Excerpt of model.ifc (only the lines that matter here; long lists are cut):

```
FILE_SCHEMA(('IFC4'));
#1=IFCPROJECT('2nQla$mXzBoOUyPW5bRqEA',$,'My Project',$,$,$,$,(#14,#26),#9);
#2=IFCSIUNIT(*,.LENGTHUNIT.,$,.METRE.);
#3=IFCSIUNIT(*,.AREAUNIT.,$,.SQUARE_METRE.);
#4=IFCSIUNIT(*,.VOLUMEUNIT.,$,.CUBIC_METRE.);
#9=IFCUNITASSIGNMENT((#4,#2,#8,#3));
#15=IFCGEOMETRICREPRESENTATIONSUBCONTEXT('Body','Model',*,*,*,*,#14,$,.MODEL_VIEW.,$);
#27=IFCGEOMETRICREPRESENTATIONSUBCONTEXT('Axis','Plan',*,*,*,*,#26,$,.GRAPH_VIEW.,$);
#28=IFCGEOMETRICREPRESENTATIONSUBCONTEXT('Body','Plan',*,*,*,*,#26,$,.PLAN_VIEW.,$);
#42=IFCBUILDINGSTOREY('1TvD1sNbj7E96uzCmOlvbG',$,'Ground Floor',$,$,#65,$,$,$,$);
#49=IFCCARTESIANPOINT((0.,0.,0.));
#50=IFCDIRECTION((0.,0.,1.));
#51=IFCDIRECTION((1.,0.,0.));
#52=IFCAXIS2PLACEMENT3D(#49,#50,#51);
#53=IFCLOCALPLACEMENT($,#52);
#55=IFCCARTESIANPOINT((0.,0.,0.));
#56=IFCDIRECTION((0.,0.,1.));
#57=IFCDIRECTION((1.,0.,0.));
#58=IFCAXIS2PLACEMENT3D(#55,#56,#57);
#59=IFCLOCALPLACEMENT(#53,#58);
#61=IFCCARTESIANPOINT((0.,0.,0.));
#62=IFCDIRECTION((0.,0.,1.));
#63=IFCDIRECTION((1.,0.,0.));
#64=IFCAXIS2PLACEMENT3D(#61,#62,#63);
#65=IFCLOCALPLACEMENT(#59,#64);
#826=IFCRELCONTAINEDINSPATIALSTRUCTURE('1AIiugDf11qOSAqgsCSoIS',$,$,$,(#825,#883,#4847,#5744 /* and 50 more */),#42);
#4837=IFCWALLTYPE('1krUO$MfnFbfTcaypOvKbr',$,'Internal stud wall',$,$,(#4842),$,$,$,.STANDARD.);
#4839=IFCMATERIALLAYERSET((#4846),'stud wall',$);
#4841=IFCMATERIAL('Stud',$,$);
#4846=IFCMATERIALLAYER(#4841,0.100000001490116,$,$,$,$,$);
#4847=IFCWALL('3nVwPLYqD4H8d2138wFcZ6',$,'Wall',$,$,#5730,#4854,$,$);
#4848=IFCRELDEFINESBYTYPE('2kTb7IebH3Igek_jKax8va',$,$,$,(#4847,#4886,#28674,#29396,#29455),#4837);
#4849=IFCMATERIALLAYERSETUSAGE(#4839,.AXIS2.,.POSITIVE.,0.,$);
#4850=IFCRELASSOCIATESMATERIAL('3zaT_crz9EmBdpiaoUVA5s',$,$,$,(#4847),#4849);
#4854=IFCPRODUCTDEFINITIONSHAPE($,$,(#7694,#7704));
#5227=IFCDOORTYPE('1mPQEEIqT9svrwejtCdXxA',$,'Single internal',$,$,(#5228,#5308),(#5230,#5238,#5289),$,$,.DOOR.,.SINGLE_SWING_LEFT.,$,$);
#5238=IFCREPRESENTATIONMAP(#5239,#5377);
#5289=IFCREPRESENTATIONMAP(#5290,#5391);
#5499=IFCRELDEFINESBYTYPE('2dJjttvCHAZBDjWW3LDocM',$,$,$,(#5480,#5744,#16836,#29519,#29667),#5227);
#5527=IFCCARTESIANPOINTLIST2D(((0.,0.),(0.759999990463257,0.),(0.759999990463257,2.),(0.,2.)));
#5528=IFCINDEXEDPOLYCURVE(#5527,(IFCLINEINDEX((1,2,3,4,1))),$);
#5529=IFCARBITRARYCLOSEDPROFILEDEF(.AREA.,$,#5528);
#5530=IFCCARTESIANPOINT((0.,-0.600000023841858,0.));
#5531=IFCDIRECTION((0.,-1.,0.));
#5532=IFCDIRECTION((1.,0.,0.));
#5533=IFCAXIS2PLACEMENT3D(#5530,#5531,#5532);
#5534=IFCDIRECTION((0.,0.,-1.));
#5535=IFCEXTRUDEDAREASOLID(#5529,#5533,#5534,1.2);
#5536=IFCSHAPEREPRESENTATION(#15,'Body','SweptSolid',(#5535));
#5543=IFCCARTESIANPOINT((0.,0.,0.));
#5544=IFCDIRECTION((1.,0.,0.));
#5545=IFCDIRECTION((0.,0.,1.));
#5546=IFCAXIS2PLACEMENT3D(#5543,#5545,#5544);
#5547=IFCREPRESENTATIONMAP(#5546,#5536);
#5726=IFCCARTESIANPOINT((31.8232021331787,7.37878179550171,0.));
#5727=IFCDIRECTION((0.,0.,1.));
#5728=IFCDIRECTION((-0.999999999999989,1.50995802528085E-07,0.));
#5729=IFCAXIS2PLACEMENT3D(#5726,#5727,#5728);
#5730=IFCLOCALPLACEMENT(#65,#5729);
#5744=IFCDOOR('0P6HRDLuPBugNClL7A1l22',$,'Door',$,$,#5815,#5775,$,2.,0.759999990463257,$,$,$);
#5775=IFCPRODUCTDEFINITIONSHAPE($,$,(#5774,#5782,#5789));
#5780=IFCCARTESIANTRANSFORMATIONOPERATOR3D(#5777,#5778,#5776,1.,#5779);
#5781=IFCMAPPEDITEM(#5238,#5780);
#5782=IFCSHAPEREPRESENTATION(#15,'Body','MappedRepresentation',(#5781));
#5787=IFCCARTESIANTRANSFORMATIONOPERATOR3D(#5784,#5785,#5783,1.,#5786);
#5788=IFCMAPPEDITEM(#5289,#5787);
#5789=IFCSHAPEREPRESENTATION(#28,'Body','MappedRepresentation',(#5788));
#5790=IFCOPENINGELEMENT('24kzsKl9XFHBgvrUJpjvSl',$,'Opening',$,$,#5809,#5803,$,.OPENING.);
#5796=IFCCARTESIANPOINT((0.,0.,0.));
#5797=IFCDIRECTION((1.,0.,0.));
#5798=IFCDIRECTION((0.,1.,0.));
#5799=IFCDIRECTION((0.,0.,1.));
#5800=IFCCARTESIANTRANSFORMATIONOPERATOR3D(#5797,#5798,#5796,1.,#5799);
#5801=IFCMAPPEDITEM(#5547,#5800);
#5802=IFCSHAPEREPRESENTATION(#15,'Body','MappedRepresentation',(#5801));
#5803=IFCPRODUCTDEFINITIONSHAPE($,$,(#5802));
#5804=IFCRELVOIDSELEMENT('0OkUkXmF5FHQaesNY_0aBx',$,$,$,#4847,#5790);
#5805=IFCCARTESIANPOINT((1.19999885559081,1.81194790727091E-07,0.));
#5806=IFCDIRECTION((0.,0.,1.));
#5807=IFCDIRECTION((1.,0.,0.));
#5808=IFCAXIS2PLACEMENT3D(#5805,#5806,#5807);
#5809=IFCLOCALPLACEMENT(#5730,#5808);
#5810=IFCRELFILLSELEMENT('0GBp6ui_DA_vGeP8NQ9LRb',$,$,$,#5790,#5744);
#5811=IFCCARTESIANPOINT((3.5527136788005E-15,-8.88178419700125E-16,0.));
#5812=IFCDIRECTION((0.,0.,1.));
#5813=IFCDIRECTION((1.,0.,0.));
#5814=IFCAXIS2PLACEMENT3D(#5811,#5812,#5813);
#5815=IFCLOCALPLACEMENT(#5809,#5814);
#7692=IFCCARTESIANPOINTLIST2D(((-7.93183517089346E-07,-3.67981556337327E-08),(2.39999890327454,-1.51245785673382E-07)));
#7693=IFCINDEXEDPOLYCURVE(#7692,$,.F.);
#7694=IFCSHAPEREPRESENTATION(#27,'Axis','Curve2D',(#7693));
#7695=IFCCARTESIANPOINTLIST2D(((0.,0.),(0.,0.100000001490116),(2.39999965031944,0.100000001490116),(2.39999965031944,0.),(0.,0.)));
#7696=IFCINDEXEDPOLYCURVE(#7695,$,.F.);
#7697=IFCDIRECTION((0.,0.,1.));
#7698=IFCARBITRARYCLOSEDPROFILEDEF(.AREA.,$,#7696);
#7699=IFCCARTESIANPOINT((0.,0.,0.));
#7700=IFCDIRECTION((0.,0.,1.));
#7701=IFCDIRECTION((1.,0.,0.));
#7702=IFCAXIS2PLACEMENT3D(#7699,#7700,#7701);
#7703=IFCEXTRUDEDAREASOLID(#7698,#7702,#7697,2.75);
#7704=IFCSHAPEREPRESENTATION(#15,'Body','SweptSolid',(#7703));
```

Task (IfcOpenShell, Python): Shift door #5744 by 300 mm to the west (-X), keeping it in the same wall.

```python
import ifcopenshell
import ifcopenshell.api.geometry
import ifcopenshell.util.placement
import ifcopenshell.util.unit

model = ifcopenshell.open("model.ifc")
unit_scale = ifcopenshell.util.unit.calculate_unit_scale(model)

door = model.by_guid("0P6HRDLuPBugNClL7A1l22")
opening = door.FillsVoids[0].RelatingOpeningElement
wall = opening.VoidsElements[0].RelatingBuildingElement

wall_matrix = ifcopenshell.util.placement.get_local_placement(wall.ObjectPlacement)
shift = wall_matrix[:3, 0] * 0.3 / unit_scale
before = ifcopenshell.util.placement.get_local_placement(door.ObjectPlacement)[:3, 3].copy()

# The door is placed relative to its opening, so it follows when the opening moves.
matrix = ifcopenshell.util.placement.get_local_placement(opening.ObjectPlacement)
matrix[:3, 3] += shift
ifcopenshell.api.geometry.edit_object_placement(
    model, product=opening, matrix=matrix, is_si=False, should_transform_children=True
)

after = ifcopenshell.util.placement.get_local_placement(door.ObjectPlacement)[:3, 3]
print("door moved by", (after - before).round(3) + 0.0)

model.write("model_edited.ifc")
```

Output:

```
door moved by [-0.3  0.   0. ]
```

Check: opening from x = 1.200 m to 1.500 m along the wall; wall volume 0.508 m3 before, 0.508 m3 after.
